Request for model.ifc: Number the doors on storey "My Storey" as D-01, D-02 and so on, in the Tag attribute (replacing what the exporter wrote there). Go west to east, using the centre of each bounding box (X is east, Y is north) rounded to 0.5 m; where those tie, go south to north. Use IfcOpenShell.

First a look at what the model holds.

```python
import ifcopenshell
import ifcopenshell.util.element
import ifcopenshell.util.placement

model = ifcopenshell.open("model.ifc")
print(model.schema)
storey = next(s for s in model.by_type("IfcBuildingStorey") if s.Name == "My Storey")
doors = [e for e in ifcopenshell.util.element.get_decomposition(storey) if e.is_a("IfcDoor")]
for e in sorted(doors, key=lambda e: e.id()):
    origin = ifcopenshell.util.placement.get_local_placement(e.ObjectPlacement)[:3, 3]
    print(e.id(), e.Tag, e.Name, origin.round(2) + 0.0, sep=" | ")
```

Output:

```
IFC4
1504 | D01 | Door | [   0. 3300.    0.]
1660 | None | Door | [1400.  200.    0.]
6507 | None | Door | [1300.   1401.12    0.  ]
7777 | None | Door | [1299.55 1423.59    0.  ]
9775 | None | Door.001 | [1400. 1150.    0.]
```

```python
import ifcopenshell
import ifcopenshell.geom
import ifcopenshell.util.element
import ifcopenshell.util.shape

model = ifcopenshell.open("model.ifc")
settings = ifcopenshell.geom.settings()
settings.set("use-world-coords", True)


def centre(element):
    shape = ifcopenshell.geom.create_shape(settings, element)
    return ifcopenshell.util.shape.get_bbox_centroid(shape.geometry)


storey = next(s for s in model.by_type("IfcBuildingStorey") if s.Name == "My Storey")
doors = [e for e in ifcopenshell.util.element.get_decomposition(storey) if e.is_a("IfcDoor")]

# Insertion points can sit at a corner or the storey origin, so sort by the geometry (in metres).
centres = {e: centre(e) for e in doors}
doors.sort(key=lambda e: (round(centres[e][0] / 0.5), centres[e][1]))

for i, e in enumerate(doors, start=1):
    number = f"D-{i:02d}"
    e.Tag = number
    print(e.id(), number)

model.write("model-out.ifc")
```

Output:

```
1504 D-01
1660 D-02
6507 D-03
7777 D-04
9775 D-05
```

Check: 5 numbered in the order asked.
